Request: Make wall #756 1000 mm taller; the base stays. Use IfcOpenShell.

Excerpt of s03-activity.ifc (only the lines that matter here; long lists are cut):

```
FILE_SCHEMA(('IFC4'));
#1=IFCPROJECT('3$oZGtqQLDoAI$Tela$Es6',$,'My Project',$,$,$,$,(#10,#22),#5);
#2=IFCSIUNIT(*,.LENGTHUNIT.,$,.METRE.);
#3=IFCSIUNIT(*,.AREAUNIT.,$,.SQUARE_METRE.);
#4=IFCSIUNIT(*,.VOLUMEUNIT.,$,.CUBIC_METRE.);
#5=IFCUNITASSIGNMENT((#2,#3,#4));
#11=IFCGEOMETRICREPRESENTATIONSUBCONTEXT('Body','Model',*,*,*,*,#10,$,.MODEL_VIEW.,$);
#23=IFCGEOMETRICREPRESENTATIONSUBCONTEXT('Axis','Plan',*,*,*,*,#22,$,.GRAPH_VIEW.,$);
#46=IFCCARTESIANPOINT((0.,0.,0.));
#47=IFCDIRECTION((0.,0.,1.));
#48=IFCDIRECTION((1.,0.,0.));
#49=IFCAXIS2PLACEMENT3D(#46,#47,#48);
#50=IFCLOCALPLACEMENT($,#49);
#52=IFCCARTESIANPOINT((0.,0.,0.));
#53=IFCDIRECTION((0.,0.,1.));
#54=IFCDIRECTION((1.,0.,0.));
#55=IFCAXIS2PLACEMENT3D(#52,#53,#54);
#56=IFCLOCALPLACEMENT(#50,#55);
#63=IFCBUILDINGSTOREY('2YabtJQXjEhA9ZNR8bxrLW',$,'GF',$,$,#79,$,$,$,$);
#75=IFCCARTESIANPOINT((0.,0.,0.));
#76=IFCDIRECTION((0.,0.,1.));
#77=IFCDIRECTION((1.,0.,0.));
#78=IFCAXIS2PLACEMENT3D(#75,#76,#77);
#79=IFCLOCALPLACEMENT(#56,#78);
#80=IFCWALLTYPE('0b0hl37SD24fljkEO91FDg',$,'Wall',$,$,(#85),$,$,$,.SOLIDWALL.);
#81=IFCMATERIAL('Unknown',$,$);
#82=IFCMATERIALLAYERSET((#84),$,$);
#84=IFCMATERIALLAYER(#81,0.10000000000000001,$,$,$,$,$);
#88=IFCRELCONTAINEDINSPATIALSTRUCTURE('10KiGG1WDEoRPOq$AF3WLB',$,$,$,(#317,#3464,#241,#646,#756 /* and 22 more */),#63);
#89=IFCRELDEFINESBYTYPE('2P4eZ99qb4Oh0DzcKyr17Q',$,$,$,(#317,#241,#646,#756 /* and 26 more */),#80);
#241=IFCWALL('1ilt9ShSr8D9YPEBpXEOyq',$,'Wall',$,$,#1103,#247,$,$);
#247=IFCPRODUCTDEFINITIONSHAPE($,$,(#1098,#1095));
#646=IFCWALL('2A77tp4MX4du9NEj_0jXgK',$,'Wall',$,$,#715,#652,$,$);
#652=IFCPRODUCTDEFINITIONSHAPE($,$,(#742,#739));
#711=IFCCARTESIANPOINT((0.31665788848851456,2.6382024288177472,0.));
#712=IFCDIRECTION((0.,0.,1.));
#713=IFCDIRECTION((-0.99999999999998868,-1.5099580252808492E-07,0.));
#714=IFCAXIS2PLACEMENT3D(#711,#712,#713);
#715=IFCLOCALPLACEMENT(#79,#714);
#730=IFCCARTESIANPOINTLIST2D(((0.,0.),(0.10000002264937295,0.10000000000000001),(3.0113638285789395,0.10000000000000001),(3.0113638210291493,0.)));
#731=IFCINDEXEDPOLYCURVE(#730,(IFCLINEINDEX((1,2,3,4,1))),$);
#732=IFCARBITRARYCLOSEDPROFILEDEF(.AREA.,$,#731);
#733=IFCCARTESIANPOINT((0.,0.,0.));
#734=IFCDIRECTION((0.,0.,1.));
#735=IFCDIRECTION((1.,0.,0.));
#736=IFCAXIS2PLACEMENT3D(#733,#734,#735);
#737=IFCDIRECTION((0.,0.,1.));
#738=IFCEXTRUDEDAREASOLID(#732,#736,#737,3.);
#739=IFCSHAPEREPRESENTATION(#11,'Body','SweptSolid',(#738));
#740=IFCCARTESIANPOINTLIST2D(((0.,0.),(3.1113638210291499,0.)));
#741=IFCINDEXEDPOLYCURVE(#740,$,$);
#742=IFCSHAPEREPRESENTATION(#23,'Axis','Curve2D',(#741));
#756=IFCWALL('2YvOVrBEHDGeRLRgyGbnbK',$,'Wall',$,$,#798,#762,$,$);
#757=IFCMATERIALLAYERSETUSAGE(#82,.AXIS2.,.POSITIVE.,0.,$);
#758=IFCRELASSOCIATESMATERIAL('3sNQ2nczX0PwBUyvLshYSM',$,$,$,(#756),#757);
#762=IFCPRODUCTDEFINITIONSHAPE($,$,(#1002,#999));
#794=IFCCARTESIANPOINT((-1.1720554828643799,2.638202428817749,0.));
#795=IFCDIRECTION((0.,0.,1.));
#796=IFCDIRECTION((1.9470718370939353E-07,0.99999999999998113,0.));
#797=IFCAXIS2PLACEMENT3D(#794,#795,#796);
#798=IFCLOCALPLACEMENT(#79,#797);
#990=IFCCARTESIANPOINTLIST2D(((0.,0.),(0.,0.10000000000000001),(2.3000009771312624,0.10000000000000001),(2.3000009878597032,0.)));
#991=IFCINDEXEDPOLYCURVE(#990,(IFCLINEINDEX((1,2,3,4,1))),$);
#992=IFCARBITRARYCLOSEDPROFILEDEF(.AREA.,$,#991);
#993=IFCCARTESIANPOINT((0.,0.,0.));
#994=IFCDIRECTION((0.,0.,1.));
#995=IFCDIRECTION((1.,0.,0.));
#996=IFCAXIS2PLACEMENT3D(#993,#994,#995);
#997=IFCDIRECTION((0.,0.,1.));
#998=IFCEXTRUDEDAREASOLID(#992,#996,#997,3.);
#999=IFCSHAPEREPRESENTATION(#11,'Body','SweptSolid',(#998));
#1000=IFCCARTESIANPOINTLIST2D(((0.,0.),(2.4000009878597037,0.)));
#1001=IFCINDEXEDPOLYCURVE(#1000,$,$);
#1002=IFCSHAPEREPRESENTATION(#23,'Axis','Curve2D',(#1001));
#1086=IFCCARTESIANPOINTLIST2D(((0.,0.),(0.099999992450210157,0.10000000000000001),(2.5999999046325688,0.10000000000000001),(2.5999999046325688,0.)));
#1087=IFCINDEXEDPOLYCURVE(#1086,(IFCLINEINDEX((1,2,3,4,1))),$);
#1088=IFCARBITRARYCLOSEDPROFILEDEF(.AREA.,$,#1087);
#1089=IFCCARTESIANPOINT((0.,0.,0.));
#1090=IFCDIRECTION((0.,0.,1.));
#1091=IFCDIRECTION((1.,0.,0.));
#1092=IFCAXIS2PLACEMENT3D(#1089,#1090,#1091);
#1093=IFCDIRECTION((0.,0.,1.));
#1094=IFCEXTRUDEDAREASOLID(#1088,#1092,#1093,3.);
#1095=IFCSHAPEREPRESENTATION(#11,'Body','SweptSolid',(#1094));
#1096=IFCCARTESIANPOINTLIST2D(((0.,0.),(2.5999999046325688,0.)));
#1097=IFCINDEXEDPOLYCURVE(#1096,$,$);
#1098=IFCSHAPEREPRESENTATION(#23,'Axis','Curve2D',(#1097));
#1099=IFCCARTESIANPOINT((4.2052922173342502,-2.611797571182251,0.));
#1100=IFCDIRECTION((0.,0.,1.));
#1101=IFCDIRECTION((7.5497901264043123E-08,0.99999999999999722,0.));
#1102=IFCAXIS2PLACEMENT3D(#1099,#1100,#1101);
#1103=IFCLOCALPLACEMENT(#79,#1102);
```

```python
import ifcopenshell
import ifcopenshell.geom
import ifcopenshell.util.representation
import ifcopenshell.util.shape
import ifcopenshell.util.unit

model = ifcopenshell.open("s03-activity.ifc")
unit_scale = ifcopenshell.util.unit.calculate_unit_scale(model)
settings = ifcopenshell.geom.settings()


def volume(element):
    """Net volume in cubic metres, openings subtracted."""
    shape = ifcopenshell.geom.create_shape(settings, element)
    return ifcopenshell.util.shape.get_volume(shape.geometry)


wall = model.by_id(756)
before = volume(wall)

body = ifcopenshell.util.representation.get_representation(wall, "Model", "Body")
solid = body.Items[0]
old_height = solid.Depth
solid.Depth += 1 / unit_scale
after = volume(wall)

print(f"height {old_height:g} -> {solid.Depth:g}, volume {before:.3f} -> {after:.3f} m3")

model.write("s03-activity_edited.ifc")
```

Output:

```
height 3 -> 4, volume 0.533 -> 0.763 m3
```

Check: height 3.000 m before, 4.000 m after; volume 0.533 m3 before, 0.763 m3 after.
